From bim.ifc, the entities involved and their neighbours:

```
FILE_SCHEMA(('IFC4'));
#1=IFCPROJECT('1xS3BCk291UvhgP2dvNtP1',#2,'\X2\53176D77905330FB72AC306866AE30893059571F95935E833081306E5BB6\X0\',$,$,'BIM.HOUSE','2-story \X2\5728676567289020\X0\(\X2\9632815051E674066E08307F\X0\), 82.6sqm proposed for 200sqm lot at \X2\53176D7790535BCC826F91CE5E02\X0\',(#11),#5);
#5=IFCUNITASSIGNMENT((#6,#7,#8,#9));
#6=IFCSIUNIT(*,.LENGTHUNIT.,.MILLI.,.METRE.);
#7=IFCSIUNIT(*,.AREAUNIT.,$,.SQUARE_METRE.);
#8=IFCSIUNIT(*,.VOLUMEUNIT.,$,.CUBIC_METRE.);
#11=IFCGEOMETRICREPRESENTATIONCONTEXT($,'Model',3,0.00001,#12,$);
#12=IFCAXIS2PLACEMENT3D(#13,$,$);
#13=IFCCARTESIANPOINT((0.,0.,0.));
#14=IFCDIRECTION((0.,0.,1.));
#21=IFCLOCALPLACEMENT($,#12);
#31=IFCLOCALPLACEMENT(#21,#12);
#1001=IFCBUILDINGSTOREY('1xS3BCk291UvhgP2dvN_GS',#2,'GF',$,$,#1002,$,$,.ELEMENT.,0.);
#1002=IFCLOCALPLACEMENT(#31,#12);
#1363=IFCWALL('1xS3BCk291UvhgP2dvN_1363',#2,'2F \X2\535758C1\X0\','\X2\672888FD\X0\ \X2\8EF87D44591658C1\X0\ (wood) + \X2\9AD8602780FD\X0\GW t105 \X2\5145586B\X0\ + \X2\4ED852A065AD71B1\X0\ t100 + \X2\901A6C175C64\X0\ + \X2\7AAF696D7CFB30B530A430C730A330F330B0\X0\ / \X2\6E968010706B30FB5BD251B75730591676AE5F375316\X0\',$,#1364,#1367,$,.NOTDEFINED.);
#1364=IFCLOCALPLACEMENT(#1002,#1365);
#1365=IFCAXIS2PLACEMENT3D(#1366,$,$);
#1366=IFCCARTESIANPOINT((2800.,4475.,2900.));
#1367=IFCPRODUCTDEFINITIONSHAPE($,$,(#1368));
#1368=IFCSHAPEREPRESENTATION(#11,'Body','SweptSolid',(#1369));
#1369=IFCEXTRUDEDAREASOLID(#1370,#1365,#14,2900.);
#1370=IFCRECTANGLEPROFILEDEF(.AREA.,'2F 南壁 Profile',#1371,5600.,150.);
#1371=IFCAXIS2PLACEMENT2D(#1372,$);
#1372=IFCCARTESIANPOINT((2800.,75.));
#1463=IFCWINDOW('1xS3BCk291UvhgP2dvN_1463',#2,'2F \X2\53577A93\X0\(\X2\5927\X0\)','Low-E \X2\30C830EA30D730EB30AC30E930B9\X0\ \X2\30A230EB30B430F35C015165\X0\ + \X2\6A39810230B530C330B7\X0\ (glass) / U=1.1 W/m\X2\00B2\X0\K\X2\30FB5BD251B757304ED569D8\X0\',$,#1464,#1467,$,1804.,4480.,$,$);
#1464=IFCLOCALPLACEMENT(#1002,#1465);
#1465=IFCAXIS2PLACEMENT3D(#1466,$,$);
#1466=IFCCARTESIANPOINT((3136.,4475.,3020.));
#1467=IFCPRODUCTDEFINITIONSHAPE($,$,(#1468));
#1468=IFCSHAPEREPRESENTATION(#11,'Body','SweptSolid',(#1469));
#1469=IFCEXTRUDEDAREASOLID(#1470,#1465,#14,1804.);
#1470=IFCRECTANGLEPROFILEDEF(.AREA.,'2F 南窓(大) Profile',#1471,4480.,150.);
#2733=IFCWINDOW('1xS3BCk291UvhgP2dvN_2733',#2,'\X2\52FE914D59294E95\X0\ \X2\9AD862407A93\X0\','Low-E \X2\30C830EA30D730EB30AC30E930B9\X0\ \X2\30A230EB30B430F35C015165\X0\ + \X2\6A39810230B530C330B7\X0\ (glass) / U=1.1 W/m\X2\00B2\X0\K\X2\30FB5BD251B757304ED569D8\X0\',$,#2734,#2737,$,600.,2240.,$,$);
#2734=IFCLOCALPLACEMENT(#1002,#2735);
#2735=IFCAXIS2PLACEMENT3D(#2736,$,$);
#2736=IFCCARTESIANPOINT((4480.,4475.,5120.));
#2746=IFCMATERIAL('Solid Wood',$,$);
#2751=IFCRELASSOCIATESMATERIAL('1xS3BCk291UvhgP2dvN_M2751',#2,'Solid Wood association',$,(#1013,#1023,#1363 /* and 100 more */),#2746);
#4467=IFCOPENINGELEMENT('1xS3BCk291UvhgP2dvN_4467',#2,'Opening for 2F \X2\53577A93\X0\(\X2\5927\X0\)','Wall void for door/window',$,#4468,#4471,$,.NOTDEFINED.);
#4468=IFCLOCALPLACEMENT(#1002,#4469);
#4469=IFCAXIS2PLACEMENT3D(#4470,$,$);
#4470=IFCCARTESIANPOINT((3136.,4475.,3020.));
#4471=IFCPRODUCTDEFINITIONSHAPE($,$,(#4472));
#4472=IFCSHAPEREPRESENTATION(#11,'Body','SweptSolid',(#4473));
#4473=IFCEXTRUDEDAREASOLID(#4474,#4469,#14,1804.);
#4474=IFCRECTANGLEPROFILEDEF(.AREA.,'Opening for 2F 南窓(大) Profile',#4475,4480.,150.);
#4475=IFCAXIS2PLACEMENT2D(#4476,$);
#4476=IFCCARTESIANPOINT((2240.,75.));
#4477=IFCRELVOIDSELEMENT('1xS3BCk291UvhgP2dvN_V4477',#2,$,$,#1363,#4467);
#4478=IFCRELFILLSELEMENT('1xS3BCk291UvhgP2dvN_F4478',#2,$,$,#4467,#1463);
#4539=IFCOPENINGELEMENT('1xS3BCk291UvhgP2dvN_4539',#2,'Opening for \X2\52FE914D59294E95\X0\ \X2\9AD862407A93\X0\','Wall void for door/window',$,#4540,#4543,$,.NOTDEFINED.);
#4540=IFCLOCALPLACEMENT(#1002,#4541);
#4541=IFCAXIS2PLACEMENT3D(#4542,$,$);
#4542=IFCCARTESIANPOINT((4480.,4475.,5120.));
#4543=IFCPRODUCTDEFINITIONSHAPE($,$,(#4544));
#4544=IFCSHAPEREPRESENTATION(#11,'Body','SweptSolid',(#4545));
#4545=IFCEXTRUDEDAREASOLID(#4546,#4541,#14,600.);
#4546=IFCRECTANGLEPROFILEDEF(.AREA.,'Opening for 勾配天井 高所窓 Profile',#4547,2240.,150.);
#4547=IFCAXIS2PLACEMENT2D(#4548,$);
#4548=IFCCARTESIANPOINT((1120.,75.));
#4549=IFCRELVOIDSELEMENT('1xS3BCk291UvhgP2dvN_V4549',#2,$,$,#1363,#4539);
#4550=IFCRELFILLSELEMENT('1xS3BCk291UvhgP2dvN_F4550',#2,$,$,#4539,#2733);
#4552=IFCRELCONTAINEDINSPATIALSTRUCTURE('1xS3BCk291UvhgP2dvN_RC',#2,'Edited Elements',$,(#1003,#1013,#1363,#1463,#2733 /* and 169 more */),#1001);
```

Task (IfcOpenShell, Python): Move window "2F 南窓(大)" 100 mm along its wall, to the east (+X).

```python
import ifcopenshell
import ifcopenshell.api.geometry
import ifcopenshell.util.placement

model = ifcopenshell.open("bim.ifc")

window = model.by_guid("1xS3BCk291UvhgP2dvN_1463")
opening = window.FillsVoids[0].RelatingOpeningElement
wall = opening.VoidsElements[0].RelatingBuildingElement

wall_matrix = ifcopenshell.util.placement.get_local_placement(wall.ObjectPlacement)
shift = wall_matrix[:3, 0] * 100.0
before = ifcopenshell.util.placement.get_local_placement(window.ObjectPlacement)[:3, 3].copy()

# The window is not placed relative to its opening, so move both.
for product in (opening, window):
    matrix = ifcopenshell.util.placement.get_local_placement(product.ObjectPlacement)
    matrix[:3, 3] += shift
    ifcopenshell.api.geometry.edit_object_placement(model, product=product, matrix=matrix, is_si=False)

after = ifcopenshell.util.placement.get_local_placement(window.ObjectPlacement)[:3, 3]
print("window moved by", (after - before).round(3) + 0.0)

model.write("bim_edited.ifc")
```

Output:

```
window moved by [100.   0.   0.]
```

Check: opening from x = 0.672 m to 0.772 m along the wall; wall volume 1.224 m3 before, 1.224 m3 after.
